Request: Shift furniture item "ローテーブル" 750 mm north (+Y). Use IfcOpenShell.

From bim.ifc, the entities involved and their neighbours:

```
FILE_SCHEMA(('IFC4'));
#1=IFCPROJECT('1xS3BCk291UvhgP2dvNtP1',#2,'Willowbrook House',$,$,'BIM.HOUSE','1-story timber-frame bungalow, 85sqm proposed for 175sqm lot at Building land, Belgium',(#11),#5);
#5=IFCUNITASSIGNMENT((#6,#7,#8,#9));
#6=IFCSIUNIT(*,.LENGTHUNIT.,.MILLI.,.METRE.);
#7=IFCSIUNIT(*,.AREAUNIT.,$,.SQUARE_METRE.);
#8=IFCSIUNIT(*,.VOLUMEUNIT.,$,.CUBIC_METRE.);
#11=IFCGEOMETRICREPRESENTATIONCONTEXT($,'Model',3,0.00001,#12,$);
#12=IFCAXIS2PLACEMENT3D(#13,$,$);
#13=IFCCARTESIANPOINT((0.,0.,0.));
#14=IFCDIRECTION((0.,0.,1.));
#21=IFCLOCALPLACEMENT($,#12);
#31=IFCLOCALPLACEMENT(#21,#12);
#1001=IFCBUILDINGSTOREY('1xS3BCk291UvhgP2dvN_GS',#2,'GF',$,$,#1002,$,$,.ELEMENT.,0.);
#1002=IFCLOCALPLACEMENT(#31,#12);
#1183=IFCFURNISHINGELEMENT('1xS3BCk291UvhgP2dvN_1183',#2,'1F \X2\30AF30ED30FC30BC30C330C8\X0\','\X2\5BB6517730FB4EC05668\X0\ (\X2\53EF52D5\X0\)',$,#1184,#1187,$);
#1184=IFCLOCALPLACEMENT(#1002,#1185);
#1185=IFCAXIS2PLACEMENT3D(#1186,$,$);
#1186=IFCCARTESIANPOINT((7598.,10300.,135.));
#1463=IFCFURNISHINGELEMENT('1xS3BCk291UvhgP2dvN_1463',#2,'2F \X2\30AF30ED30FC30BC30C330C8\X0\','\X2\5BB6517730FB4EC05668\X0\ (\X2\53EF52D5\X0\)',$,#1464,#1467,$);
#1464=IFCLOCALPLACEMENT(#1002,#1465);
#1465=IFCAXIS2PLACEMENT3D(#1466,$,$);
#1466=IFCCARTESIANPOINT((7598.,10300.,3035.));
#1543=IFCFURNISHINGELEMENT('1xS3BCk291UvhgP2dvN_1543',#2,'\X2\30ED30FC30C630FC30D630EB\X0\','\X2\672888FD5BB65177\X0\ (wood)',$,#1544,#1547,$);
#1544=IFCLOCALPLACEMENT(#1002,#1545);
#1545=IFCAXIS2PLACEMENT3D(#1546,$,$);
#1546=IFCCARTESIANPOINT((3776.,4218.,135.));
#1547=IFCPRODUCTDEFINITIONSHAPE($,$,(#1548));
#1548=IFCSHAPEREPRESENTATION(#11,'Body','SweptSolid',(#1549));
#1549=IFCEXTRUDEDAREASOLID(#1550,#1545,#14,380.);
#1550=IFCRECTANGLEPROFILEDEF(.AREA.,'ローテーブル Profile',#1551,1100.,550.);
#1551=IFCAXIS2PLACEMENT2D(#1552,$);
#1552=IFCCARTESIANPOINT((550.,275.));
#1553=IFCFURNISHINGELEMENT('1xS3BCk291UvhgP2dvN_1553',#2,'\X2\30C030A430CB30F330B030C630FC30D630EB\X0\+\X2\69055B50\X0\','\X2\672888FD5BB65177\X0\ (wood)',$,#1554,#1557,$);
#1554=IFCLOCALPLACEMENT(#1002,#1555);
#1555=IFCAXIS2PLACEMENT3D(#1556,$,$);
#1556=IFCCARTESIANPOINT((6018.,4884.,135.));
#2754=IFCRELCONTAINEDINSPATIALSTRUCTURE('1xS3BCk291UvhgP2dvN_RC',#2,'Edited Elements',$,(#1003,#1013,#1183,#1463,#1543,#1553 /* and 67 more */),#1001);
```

```python
import ifcopenshell
import ifcopenshell.api.geometry
import ifcopenshell.util.placement
import ifcopenshell.util.unit

model = ifcopenshell.open("bim.ifc")
unit_scale = ifcopenshell.util.unit.calculate_unit_scale(model)

item = model.by_id(1543)
matrix = ifcopenshell.util.placement.get_local_placement(item.ObjectPlacement)
matrix[1, 3] += 0.75 / unit_scale
ifcopenshell.api.geometry.edit_object_placement(model, product=item, matrix=matrix, is_si=False)

print(ifcopenshell.util.placement.get_local_placement(item.ObjectPlacement).round(3) + 0.0)

model.write("bim-out.ifc")
```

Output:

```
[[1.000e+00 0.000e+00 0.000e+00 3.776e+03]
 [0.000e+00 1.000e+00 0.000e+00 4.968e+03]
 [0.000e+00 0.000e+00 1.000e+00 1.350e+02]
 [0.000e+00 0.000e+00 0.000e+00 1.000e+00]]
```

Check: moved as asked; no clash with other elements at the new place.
